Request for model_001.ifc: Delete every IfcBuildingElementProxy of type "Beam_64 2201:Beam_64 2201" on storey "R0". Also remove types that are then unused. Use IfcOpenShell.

First a look at what the model holds.

```python
import ifcopenshell
import ifcopenshell.util.element

model = ifcopenshell.open("model_001.ifc")
print(model.schema)
storey = next(s for s in model.by_type("IfcBuildingStorey") if s.Name == "R0")
proxies = [e for e in ifcopenshell.util.element.get_decomposition(storey) if e.is_a("IfcBuildingElementProxy")]
seen = {}
for e in proxies:
    element_type = ifcopenshell.util.element.get_type(e)
    name = element_type.Name if element_type not in (None, e) else None
    seen[name] = seen.get(name, 0) + 1
for name, count in sorted(seen.items(), key=str):
    print(count, "x", name)
```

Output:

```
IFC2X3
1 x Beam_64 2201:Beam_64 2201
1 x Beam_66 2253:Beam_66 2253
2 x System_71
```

```python
import ifcopenshell
import ifcopenshell.api.root
import ifcopenshell.util.element

model = ifcopenshell.open("model_001.ifc")

storey = next(s for s in model.by_type("IfcBuildingStorey") if s.Name == "R0")
proxies = [e for e in ifcopenshell.util.element.get_decomposition(storey) if e.is_a("IfcBuildingElementProxy")]
targets = [e for e in proxies if (t := ifcopenshell.util.element.get_type(e)) not in (None, e) and t.Name == "Beam_64 2201:Beam_64 2201"]
types = {ifcopenshell.util.element.get_type(e) for e in targets} - {None, *targets}

for e in targets:
    ifcopenshell.api.root.remove_product(model, product=e)
print(len(targets), "removed")

unused = [t for t in types if not ifcopenshell.util.element.get_types(t)]
for t in unused:
    ifcopenshell.api.root.remove_product(model, product=t)
print(len(unused), "unused types removed")

model.write("model_001-out.ifc")
```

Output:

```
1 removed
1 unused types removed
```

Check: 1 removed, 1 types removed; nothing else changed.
